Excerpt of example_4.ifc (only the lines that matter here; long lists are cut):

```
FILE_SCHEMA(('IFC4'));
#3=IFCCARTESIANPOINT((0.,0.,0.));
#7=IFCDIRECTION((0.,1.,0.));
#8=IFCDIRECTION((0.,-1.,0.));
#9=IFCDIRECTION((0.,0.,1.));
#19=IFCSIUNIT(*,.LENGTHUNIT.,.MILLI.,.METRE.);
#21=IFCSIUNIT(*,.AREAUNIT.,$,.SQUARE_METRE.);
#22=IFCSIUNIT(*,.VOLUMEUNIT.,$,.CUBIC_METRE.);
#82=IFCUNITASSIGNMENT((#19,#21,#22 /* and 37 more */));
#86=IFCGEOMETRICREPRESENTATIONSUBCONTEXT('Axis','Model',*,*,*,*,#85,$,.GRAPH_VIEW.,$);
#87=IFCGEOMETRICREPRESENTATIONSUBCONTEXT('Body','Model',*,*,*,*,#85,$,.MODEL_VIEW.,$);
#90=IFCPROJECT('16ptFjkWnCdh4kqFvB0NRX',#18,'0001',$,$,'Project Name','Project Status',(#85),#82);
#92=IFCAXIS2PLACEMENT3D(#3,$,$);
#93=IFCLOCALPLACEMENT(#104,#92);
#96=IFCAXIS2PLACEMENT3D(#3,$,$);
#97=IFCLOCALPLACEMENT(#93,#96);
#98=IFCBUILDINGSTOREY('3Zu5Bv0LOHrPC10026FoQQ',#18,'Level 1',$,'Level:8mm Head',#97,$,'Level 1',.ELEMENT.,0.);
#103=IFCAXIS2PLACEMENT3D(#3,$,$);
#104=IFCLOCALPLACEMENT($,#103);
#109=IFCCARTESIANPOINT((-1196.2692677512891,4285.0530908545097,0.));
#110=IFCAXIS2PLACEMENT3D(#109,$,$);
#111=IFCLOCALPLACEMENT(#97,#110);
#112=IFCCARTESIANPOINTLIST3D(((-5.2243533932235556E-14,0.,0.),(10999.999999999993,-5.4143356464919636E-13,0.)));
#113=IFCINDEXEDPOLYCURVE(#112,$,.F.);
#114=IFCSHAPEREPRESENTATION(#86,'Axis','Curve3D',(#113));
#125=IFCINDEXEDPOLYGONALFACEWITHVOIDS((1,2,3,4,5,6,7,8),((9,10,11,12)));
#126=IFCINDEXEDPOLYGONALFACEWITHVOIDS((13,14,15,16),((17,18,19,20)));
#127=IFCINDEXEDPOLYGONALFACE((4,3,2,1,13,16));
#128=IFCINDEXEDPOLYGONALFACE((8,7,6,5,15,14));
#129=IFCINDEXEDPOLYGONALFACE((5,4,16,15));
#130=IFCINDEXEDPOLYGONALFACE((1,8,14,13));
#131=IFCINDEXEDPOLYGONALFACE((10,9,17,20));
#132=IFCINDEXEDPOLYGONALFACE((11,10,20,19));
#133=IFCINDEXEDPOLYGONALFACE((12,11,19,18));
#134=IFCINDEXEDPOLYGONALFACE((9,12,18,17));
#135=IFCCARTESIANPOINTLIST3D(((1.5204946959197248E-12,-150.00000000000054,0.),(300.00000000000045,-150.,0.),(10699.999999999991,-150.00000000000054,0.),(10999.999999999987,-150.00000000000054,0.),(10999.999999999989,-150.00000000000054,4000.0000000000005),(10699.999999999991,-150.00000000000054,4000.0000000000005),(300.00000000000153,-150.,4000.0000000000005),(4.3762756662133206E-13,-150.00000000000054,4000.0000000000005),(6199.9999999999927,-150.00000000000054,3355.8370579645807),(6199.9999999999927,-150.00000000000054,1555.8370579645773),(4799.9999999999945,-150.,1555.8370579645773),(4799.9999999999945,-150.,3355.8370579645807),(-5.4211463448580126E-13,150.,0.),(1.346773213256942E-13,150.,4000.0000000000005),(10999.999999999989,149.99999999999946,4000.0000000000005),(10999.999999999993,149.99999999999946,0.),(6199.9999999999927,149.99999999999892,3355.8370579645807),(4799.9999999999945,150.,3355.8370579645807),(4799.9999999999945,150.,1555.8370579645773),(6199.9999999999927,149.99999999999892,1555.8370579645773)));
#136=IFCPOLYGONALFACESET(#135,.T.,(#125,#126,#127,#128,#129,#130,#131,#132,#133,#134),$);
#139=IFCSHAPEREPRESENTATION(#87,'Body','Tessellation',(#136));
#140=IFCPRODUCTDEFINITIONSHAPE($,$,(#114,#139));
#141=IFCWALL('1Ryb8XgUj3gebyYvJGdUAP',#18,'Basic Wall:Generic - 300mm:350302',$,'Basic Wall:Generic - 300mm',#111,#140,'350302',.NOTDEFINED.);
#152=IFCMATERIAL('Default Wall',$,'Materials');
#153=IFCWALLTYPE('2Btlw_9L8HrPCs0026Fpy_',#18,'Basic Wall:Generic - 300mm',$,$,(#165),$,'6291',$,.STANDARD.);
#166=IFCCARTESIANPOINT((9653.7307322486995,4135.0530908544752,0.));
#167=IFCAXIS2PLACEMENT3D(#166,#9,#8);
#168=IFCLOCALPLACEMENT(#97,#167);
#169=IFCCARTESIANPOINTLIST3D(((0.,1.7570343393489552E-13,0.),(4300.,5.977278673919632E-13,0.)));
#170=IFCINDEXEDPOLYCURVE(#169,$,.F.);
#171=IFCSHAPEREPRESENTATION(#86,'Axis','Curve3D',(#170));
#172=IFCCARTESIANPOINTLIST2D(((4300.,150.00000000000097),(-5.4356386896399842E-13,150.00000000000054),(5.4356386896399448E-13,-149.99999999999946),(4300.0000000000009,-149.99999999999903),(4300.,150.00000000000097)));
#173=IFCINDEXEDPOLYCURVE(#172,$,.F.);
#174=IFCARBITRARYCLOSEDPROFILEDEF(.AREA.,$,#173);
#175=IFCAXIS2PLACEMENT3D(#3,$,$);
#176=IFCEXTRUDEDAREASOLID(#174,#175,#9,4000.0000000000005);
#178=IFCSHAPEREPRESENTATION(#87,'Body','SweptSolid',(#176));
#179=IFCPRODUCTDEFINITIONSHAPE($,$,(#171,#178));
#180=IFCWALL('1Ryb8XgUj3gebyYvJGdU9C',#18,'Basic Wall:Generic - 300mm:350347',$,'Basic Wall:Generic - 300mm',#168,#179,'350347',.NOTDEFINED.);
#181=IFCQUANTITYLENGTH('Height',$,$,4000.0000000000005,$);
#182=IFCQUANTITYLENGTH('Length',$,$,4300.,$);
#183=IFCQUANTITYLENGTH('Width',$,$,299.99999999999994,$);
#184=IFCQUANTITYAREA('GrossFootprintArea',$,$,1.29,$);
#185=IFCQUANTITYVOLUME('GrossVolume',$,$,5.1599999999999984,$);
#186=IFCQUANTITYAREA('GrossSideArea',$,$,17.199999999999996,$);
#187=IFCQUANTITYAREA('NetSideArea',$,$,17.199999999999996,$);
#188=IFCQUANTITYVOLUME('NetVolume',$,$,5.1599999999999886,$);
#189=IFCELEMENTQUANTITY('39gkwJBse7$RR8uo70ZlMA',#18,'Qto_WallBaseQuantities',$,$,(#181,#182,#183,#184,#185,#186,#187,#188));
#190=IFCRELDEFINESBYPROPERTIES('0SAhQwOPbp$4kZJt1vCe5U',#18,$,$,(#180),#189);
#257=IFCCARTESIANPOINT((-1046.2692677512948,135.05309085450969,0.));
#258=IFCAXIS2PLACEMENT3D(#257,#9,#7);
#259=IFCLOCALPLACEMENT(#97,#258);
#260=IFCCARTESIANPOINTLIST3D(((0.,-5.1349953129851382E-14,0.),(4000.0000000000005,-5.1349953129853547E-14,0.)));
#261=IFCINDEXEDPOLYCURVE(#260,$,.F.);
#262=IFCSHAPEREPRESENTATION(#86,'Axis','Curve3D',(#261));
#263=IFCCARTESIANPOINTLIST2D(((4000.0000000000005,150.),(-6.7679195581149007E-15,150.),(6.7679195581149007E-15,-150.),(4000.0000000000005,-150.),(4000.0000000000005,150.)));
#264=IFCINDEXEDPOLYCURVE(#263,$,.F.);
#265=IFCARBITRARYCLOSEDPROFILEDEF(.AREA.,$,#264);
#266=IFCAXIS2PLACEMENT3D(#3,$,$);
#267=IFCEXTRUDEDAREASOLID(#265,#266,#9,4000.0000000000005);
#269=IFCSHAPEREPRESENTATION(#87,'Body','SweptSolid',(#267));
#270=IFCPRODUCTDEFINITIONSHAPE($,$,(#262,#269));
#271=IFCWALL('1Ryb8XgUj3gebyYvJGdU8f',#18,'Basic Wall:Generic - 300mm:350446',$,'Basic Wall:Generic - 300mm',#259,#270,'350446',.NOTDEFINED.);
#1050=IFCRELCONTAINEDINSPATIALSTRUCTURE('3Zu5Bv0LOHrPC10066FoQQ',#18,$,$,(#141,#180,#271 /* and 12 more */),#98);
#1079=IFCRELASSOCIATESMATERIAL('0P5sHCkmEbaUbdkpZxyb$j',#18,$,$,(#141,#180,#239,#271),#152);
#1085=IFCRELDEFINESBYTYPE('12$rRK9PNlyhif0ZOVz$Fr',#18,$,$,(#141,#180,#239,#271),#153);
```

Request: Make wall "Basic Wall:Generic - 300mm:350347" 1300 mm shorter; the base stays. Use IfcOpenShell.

```python
import ifcopenshell
import ifcopenshell.api.pset
import ifcopenshell.geom
import ifcopenshell.util.element
import ifcopenshell.util.representation
import ifcopenshell.util.shape
import ifcopenshell.util.unit

model = ifcopenshell.open("example_4.ifc")
unit_scale = ifcopenshell.util.unit.calculate_unit_scale(model)
area_scale = ifcopenshell.util.unit.calculate_unit_scale(model, "AREAUNIT")
volume_scale = ifcopenshell.util.unit.calculate_unit_scale(model, "VOLUMEUNIT")
settings = ifcopenshell.geom.settings()


def volume(element):
    """Net volume in cubic metres, openings subtracted."""
    shape = ifcopenshell.geom.create_shape(settings, element)
    return ifcopenshell.util.shape.get_volume(shape.geometry)


wall = model.by_id(180)
before = volume(wall)

body = ifcopenshell.util.representation.get_representation(wall, "Model", "Body")
solid = body.Items[0]
old_height = solid.Depth
solid.Depth -= 1300.0
after = volume(wall)
thickness = 0.3  # wall thickness in metres

# Update the stored height, areas and volumes.
qto = model.by_id(ifcopenshell.util.element.get_pset(wall, "Qto_WallBaseQuantities", should_inherit=False)["id"])
ifcopenshell.api.pset.edit_qto(model, qto=qto, properties={
    "Height": solid.Depth,
    "GrossVolume": ifcopenshell.util.element.get_pset(wall, "Qto_WallBaseQuantities", "GrossVolume") * solid.Depth / old_height,
    "GrossSideArea": ifcopenshell.util.element.get_pset(wall, "Qto_WallBaseQuantities", "GrossSideArea") * solid.Depth / old_height,
    "NetSideArea": after / thickness / area_scale,
    "NetVolume": after / volume_scale,
})

print(f"height {old_height:g} -> {solid.Depth:g}, volume {before:.3f} -> {after:.3f} m3")

model.write("example_4_v2.ifc")
```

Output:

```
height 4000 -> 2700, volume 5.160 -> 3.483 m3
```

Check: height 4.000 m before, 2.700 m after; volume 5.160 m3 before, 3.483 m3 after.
